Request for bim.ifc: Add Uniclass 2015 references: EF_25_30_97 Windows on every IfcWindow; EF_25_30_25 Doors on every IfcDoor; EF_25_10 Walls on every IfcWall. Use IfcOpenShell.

First a look at what the model holds.

```python
import ifcopenshell

model = ifcopenshell.open("bim.ifc")
print(model.schema)
print("classifications:", [c.Name for c in model.by_type("IfcClassification")])
for ifc_class in ("IfcDoor", "IfcRoof", "IfcStair", "IfcWall", "IfcWindow"):
    print(ifc_class, len(model.by_type(ifc_class)))
```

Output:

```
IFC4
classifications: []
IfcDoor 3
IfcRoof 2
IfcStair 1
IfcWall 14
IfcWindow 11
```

```python
import ifcopenshell
import ifcopenshell.api.classification

model = ifcopenshell.open("bim.ifc")

system = ifcopenshell.api.classification.add_classification(model, classification="Uniclass 2015")

codes = {
    "IfcWindow": ("EF_25_30_97", "Windows"),
    "IfcDoor": ("EF_25_30_25", "Doors"),
    "IfcWall": ("EF_25_10", "Walls"),
}
for ifc_class, (code, name) in codes.items():
    products = model.by_type(ifc_class)
    ifcopenshell.api.classification.add_reference(
        model, products=products, classification=system, identification=code, name=name
    )
    print(code, len(products))

model.write("bim_edited.ifc")
```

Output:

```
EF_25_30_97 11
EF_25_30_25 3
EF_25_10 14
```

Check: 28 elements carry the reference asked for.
